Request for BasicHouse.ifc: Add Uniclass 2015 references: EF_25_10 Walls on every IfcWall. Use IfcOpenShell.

First a look at what the model holds.

```python
import ifcopenshell

model = ifcopenshell.open("BasicHouse.ifc")
print(model.schema)
print("classifications:", [c.Name for c in model.by_type("IfcClassification")])
for ifc_class in ("IfcDoor", "IfcRoof", "IfcStair", "IfcWall", "IfcWindow"):
    print(ifc_class, len(model.by_type(ifc_class)))
```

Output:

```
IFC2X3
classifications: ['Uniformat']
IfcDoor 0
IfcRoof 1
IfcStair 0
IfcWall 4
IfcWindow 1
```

```python
import ifcopenshell
import ifcopenshell.api.classification

model = ifcopenshell.open("BasicHouse.ifc")

# IFC2X3 requires Source and Edition and has no link from the project to the system.
system = model.create_entity("IfcClassification", Source="NBS", Edition="2015", Name="Uniclass 2015")

codes = {
    "IfcWall": ("EF_25_10", "Walls"),
}
for ifc_class, (code, name) in codes.items():
    products = model.by_type(ifc_class)
    ifcopenshell.api.classification.add_reference(
        model, products=products, classification=system, identification=code, name=name
    )
    print(code, len(products))

model.write("BasicHouse_updated.ifc")
```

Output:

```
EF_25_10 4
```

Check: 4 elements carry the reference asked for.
